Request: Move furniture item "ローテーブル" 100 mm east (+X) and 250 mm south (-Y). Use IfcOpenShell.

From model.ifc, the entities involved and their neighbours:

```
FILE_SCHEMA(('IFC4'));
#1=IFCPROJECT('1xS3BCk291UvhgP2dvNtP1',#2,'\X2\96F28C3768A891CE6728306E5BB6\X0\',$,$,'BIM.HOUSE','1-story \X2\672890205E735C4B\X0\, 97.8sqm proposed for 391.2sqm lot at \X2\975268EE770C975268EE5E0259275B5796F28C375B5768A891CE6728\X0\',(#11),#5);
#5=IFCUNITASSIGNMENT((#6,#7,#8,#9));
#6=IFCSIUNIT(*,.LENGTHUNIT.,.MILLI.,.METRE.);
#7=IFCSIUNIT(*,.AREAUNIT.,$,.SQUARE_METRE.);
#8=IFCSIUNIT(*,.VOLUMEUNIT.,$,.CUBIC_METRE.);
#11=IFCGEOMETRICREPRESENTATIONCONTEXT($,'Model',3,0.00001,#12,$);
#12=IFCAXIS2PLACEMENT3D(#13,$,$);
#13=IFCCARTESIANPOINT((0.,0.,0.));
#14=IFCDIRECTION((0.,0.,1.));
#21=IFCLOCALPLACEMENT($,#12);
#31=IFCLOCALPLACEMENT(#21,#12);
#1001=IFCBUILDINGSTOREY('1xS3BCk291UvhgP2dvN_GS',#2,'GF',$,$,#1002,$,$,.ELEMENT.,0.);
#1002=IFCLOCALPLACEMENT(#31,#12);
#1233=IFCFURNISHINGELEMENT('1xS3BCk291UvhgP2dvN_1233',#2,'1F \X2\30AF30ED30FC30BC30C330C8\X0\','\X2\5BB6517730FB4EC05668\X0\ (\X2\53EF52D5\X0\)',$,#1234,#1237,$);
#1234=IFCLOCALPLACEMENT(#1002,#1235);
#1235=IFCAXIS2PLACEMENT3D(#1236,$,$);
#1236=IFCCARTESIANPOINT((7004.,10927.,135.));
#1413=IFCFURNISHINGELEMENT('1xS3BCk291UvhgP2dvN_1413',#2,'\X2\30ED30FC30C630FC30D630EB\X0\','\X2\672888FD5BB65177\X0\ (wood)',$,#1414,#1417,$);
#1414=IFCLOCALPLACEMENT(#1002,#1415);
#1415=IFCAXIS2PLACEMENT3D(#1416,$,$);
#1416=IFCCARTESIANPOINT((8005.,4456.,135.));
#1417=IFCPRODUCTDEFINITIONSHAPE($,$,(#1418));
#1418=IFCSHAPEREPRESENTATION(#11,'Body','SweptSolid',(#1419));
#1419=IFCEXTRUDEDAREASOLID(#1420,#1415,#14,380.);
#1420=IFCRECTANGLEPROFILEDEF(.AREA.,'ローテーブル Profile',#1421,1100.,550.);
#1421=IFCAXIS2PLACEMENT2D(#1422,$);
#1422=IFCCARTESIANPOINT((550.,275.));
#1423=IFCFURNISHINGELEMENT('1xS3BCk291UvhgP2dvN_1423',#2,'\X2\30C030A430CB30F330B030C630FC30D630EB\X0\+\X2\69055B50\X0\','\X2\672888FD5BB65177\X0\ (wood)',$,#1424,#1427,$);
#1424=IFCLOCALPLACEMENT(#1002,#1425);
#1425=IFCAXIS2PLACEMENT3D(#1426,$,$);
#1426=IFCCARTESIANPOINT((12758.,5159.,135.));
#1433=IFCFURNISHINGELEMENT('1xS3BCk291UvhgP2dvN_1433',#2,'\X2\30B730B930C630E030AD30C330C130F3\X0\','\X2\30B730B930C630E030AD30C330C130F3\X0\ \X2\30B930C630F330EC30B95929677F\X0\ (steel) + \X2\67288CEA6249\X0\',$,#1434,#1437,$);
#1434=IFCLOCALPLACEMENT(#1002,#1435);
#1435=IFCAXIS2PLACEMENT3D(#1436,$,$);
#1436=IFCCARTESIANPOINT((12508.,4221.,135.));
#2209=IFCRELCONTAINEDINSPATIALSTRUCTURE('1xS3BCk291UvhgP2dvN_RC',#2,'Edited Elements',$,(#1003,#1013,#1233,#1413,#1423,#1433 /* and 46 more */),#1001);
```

```python
import ifcopenshell
import ifcopenshell.api.geometry
import ifcopenshell.util.placement

model = ifcopenshell.open("model.ifc")

item = model.by_guid("1xS3BCk291UvhgP2dvN_1413")
matrix = ifcopenshell.util.placement.get_local_placement(item.ObjectPlacement)
matrix[0, 3] += 100.0
matrix[1, 3] -= 250.0
ifcopenshell.api.geometry.edit_object_placement(model, product=item, matrix=matrix, is_si=False)

print(ifcopenshell.util.placement.get_local_placement(item.ObjectPlacement).round(3) + 0.0)

model.write("model_rev.ifc")
```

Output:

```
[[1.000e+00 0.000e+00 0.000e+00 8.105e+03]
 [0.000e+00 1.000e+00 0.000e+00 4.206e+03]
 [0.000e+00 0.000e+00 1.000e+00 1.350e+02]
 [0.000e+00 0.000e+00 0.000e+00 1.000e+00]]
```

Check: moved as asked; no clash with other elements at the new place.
